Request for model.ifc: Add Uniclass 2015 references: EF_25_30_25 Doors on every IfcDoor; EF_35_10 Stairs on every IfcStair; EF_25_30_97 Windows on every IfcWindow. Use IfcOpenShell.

First a look at what the model holds.

```python
import ifcopenshell

model = ifcopenshell.open("model.ifc")
print(model.schema)
print("classifications:", [c.Name for c in model.by_type("IfcClassification")])
for ifc_class in ("IfcDoor", "IfcRoof", "IfcStair", "IfcWall", "IfcWindow"):
    print(ifc_class, len(model.by_type(ifc_class)))
```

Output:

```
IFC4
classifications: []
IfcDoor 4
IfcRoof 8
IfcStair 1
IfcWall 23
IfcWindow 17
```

```python
import ifcopenshell
import ifcopenshell.api.classification

model = ifcopenshell.open("model.ifc")

system = ifcopenshell.api.classification.add_classification(model, classification="Uniclass 2015")

codes = {
    "IfcDoor": ("EF_25_30_25", "Doors"),
    "IfcStair": ("EF_35_10", "Stairs"),
    "IfcWindow": ("EF_25_30_97", "Windows"),
}
for ifc_class, (code, name) in codes.items():
    products = model.by_type(ifc_class)
    ifcopenshell.api.classification.add_reference(
        model, products=products, classification=system, identification=code, name=name
    )
    print(code, len(products))

model.write("model_updated.ifc")
```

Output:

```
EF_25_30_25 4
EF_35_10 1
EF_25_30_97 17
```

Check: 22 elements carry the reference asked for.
